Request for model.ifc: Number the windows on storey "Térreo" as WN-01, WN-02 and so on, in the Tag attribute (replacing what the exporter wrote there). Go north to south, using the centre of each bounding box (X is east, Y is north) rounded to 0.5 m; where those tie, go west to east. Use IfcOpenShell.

First a look at what the model holds.

```python
import ifcopenshell
import ifcopenshell.util.element
import ifcopenshell.util.placement

model = ifcopenshell.open("model.ifc")
print(model.schema)
storey = next(s for s in model.by_type("IfcBuildingStorey") if s.Name == "Térreo")
windows = [e for e in ifcopenshell.util.element.get_decomposition(storey) if e.is_a("IfcWindow")]
for e in sorted(windows, key=lambda e: e.id()):
    origin = ifcopenshell.util.placement.get_local_placement(e.ObjectPlacement)[:3, 3]
    print(e.id(), e.Tag, e.Name, origin.round(2) + 0.0, sep=" | ")
```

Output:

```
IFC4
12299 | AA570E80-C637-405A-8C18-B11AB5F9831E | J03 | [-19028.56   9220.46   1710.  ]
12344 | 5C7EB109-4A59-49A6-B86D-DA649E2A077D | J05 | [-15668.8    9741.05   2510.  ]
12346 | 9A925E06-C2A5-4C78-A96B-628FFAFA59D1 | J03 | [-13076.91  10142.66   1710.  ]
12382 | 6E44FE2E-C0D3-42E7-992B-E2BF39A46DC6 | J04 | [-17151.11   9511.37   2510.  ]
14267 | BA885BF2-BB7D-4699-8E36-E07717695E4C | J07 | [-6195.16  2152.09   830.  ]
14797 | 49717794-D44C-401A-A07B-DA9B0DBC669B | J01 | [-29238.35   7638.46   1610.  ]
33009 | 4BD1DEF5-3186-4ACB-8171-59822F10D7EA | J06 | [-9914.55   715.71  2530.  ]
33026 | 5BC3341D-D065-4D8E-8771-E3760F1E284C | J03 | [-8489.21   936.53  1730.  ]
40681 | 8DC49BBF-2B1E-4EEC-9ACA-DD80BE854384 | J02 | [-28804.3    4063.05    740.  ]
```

```python
import ifcopenshell
import ifcopenshell.geom
import ifcopenshell.util.element
import ifcopenshell.util.shape

model = ifcopenshell.open("model.ifc")
settings = ifcopenshell.geom.settings()
settings.set("use-world-coords", True)


def centre(element):
    shape = ifcopenshell.geom.create_shape(settings, element)
    return ifcopenshell.util.shape.get_bbox_centroid(shape.geometry)


storey = next(s for s in model.by_type("IfcBuildingStorey") if s.Name == "Térreo")
windows = [e for e in ifcopenshell.util.element.get_decomposition(storey) if e.is_a("IfcWindow")]

# Insertion points can sit at a corner or the storey origin, so sort by the geometry (in metres).
centres = {e: centre(e) for e in windows}
windows.sort(key=lambda e: (-round(centres[e][1] / 0.5), centres[e][0]))

for i, e in enumerate(windows, start=1):
    number = f"WN-{i:02d}"
    e.Tag = number
    print(e.id(), number)

model.write("model_edited.ifc")
```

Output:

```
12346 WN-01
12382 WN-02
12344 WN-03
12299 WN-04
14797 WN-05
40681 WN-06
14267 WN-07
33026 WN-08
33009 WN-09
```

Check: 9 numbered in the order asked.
